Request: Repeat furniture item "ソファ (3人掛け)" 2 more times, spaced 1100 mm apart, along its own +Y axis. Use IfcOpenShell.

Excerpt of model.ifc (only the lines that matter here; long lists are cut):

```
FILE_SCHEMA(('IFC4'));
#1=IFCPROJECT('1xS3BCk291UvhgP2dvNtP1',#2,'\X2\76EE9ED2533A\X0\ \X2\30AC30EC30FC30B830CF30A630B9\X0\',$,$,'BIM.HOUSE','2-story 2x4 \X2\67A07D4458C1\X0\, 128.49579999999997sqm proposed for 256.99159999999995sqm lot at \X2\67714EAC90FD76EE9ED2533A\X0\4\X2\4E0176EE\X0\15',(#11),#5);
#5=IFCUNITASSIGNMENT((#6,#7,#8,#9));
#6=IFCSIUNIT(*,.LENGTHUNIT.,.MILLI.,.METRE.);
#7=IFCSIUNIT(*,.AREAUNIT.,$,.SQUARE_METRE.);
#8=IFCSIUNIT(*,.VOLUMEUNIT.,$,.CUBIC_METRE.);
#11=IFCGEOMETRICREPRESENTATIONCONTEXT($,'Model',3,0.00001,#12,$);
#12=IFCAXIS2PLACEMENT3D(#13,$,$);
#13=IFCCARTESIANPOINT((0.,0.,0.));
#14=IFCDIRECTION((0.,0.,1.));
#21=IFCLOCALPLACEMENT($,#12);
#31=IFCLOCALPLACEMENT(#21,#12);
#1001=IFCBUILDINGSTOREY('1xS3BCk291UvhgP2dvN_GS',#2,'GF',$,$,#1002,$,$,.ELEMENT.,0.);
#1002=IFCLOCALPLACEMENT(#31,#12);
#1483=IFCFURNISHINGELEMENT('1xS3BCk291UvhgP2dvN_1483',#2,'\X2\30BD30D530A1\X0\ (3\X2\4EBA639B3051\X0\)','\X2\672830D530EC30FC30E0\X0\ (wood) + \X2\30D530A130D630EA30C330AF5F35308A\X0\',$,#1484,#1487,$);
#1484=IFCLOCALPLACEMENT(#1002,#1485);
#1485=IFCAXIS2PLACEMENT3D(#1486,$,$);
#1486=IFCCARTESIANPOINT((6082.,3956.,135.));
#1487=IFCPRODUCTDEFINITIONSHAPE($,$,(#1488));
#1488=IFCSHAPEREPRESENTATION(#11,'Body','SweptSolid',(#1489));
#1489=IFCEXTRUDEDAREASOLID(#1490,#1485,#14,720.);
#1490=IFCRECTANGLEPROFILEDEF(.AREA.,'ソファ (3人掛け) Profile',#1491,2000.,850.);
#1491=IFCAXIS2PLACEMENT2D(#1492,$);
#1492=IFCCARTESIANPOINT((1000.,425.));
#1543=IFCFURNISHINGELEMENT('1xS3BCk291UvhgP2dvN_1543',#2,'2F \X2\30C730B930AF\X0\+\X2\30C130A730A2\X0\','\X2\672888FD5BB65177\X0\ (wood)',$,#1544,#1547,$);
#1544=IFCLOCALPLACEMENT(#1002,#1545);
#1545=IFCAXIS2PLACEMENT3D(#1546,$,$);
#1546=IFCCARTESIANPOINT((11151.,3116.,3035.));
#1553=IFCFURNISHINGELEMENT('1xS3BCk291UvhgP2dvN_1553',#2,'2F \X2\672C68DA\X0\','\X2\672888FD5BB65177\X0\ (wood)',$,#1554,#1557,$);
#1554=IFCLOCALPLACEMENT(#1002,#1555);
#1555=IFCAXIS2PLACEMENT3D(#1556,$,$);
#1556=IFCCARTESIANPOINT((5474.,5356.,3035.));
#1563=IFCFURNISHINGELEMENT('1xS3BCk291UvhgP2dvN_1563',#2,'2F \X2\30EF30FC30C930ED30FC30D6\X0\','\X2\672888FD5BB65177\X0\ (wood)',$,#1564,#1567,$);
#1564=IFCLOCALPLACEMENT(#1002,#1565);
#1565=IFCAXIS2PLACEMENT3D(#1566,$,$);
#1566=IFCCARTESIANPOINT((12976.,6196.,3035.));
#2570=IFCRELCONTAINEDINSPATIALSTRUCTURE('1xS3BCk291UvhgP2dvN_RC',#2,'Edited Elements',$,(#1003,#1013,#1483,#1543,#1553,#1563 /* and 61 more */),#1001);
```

```python
import ifcopenshell
import ifcopenshell.api.geometry
import ifcopenshell.api.root
import ifcopenshell.util.element
import ifcopenshell.util.placement
import ifcopenshell.util.unit

model = ifcopenshell.open("model.ifc")
unit_scale = ifcopenshell.util.unit.calculate_unit_scale(model)


def reuse_history(source, copy):
    """copy_class also copies each property set's owner history, people and application; keep the originals."""
    for rel in copy.IsDefinedBy:
        if rel.is_a("IfcRelDefinesByProperties") and (history := rel.RelatingPropertyDefinition.OwnerHistory):
            rel.RelatingPropertyDefinition.OwnerHistory = source.OwnerHistory
            ifcopenshell.util.element.remove_deep2(model, history)


source = model.by_id(1483)
base = ifcopenshell.util.placement.get_local_placement(source.ObjectPlacement)
step = base[:3, 1] * 1.1 / unit_scale

for i in range(1, 3):
    copy = ifcopenshell.api.root.copy_class(model, product=source)
    copy.Representation = ifcopenshell.util.element.copy_deep(
        model, source.Representation, exclude=["IfcGeometricRepresentationContext", "IfcRepresentationMap"]
    )
    reuse_history(source, copy)
    matrix = base.copy()
    matrix[:3, 3] += i * step
    print("added at", matrix[:3, 3].round(3) + 0.0)
    ifcopenshell.api.geometry.edit_object_placement(model, product=copy, matrix=matrix, is_si=False)

model.write("model-out.ifc")
```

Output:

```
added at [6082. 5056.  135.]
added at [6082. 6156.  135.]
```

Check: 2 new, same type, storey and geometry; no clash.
